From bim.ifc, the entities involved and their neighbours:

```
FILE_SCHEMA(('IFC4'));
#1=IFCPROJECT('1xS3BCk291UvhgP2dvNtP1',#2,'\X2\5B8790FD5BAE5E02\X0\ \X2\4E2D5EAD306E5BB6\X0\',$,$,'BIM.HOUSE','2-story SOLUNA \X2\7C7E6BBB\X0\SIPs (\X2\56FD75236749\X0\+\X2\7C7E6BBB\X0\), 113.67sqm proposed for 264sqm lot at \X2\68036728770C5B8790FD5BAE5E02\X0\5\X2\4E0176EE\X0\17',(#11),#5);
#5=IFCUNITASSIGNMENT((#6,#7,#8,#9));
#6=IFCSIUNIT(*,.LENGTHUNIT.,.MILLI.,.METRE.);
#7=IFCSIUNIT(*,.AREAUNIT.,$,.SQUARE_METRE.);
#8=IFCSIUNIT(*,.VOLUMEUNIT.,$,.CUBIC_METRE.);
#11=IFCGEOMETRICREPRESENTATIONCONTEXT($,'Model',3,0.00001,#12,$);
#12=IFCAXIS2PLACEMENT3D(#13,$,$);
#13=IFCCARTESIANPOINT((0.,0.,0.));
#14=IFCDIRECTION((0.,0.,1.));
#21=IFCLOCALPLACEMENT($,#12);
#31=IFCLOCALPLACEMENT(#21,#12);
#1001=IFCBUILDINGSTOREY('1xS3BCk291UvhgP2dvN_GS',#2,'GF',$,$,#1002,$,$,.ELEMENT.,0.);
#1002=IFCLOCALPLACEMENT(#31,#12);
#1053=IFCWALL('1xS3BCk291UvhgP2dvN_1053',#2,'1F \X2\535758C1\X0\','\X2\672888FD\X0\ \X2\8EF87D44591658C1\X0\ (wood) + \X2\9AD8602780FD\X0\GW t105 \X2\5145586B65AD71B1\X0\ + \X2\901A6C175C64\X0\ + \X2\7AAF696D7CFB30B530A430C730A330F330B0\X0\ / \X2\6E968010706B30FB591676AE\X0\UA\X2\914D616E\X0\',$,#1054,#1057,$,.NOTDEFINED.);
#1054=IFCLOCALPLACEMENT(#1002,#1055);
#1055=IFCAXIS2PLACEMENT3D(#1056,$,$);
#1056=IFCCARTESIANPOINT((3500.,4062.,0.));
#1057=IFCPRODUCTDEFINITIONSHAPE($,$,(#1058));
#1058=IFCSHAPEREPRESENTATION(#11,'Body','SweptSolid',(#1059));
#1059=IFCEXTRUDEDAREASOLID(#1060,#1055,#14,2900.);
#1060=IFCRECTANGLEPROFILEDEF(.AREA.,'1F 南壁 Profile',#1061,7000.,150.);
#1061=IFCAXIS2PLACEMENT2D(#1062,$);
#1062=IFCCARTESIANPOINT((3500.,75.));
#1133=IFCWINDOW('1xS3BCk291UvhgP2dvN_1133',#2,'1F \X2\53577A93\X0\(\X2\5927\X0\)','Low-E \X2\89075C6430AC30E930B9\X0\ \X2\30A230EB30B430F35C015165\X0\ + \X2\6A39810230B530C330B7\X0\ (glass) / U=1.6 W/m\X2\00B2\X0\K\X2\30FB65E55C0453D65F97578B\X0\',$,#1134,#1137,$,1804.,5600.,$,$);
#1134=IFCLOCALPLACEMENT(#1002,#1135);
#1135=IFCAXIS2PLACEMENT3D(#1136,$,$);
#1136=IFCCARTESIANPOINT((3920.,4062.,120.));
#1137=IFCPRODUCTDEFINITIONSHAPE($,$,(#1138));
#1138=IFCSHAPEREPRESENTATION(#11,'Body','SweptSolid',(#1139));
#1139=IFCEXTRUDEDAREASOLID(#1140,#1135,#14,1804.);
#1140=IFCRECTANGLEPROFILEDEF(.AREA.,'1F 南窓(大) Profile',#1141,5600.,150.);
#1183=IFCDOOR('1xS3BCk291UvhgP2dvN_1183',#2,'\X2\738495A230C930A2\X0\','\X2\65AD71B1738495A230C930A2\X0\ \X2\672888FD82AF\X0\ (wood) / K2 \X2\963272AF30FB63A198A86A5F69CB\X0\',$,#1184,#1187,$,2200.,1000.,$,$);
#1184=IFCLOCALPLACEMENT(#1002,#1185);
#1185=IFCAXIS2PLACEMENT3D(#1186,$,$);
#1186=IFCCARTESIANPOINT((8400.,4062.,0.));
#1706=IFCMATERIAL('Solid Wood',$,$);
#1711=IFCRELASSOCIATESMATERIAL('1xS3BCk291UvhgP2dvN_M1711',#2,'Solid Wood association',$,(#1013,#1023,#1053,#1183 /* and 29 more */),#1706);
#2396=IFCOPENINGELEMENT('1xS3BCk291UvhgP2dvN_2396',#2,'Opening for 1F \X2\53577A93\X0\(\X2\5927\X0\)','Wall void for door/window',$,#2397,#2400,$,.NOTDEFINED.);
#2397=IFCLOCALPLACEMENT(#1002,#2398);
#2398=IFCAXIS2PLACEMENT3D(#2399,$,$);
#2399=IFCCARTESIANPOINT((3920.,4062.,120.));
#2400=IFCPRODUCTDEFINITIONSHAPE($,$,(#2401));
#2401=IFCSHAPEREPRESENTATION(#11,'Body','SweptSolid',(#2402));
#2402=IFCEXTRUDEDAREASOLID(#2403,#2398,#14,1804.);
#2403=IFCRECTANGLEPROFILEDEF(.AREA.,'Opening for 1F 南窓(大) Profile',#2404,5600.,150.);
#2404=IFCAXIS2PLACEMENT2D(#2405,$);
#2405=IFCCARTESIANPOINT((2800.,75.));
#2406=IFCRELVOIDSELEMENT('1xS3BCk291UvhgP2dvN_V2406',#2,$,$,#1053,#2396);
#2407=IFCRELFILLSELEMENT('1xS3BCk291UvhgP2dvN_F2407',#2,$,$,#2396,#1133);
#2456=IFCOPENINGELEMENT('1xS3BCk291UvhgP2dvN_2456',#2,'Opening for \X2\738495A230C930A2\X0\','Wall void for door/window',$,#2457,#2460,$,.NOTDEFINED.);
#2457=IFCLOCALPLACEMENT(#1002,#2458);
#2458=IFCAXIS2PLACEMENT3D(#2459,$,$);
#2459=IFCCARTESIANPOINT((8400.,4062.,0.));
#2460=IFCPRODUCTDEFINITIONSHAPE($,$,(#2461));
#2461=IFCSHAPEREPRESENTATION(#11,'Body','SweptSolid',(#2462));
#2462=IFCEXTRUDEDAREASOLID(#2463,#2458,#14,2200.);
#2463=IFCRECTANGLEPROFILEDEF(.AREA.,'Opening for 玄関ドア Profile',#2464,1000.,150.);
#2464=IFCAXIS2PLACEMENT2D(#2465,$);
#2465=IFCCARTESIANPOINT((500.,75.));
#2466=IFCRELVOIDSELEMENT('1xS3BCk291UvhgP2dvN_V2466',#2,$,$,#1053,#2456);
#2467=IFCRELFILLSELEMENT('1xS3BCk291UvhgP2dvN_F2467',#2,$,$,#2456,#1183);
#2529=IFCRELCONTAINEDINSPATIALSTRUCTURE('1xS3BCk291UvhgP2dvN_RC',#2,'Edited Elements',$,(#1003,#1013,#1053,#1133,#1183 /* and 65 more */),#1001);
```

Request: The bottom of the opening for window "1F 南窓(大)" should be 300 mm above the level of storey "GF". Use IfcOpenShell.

```python
import numpy as np
import ifcopenshell
import ifcopenshell.api.geometry
import ifcopenshell.geom
import ifcopenshell.util.element
import ifcopenshell.util.placement
import ifcopenshell.util.shape
import ifcopenshell.util.unit

model = ifcopenshell.open("bim.ifc")
unit_scale = ifcopenshell.util.unit.calculate_unit_scale(model)

window = model.by_id(1133)
opening = window.FillsVoids[0].RelatingOpeningElement
storey = ifcopenshell.util.element.get_container(window, ifc_class="IfcBuildingStorey")
level = ifcopenshell.util.placement.get_local_placement(storey.ObjectPlacement)[2, 3]

# The opening's origin need not be at the sill, so measure its lowest point.
shape = ifcopenshell.geom.create_shape(ifcopenshell.geom.settings(), opening)
bottom = ifcopenshell.util.shape.get_shape_bottom_elevation(shape, shape.geometry) / unit_scale
dz = level + 0.3 / unit_scale - bottom

shift = np.array([0.0, 0.0, dz])
# The window is not placed relative to its opening, so move both.
for product in (opening, window):
    matrix = ifcopenshell.util.placement.get_local_placement(product.ObjectPlacement)
    matrix[:3, 3] += shift
    ifcopenshell.api.geometry.edit_object_placement(model, product=product, matrix=matrix, is_si=False)

print(f"moved by {dz * unit_scale:+.3f} m")

model.write("bim-out.ifc")
```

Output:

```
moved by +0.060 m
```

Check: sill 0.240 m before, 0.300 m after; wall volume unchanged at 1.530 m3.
